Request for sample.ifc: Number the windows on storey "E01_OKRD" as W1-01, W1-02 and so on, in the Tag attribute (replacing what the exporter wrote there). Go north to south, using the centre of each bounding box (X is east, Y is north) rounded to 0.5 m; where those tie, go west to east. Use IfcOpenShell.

First a look at what the model holds.

```python
import ifcopenshell
import ifcopenshell.util.element
import ifcopenshell.util.placement

model = ifcopenshell.open("sample.ifc")
print(model.schema)
storey = next(s for s in model.by_type("IfcBuildingStorey") if s.Name == "E01_OKRD")
windows = [e for e in ifcopenshell.util.element.get_decomposition(storey) if e.is_a("IfcWindow")]
for e in sorted(windows, key=lambda e: e.id()):
    origin = ifcopenshell.util.placement.get_local_placement(e.ObjectPlacement)[:3, 3]
    print(e.id(), e.Tag, e.Name, origin.round(2) + 0.0, sep=" | ")
```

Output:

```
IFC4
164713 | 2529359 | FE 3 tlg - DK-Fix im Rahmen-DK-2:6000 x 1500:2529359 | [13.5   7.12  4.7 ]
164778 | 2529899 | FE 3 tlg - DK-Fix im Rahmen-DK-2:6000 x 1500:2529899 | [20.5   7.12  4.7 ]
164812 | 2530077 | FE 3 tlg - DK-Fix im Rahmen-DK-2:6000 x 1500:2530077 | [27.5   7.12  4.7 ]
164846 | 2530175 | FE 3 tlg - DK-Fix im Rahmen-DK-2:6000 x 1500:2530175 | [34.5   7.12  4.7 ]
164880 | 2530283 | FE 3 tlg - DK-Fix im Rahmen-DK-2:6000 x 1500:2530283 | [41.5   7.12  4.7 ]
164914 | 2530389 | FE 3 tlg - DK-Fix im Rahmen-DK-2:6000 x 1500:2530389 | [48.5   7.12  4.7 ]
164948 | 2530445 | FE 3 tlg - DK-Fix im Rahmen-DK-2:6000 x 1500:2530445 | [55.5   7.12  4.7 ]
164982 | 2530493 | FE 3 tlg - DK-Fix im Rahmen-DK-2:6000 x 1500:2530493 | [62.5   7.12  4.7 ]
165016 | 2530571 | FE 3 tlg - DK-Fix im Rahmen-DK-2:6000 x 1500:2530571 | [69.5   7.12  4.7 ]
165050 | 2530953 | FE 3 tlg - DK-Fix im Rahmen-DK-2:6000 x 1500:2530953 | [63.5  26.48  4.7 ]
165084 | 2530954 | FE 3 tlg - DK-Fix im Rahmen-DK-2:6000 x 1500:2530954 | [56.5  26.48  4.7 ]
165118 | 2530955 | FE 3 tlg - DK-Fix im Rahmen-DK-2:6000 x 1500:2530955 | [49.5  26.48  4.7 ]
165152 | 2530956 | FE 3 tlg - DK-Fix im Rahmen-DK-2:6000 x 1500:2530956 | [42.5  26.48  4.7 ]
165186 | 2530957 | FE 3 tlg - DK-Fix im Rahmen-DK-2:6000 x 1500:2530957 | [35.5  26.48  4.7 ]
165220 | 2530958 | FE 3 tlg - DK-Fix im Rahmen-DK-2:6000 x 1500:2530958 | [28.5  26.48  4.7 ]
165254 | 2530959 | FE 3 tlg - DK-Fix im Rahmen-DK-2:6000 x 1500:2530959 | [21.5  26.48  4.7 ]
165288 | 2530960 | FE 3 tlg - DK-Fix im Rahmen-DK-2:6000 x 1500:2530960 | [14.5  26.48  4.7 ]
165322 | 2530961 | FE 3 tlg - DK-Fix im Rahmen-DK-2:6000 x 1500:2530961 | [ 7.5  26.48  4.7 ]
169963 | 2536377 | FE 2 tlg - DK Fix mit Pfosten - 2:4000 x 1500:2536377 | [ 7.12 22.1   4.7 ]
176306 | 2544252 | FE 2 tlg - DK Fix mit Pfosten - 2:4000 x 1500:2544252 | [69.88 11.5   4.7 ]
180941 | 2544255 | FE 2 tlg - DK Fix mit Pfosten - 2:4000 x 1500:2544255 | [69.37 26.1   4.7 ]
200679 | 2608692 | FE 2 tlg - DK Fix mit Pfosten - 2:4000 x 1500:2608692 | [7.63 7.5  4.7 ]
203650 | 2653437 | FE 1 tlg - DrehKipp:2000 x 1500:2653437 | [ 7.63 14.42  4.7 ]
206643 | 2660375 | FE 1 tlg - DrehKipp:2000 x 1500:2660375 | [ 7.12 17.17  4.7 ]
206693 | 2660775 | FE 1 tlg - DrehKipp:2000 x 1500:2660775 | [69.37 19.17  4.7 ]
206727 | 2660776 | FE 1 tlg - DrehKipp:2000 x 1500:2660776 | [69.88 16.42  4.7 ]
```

```python
import ifcopenshell
import ifcopenshell.geom
import ifcopenshell.util.element
import ifcopenshell.util.shape

model = ifcopenshell.open("sample.ifc")
settings = ifcopenshell.geom.settings()
settings.set("use-world-coords", True)


def centre(element):
    shape = ifcopenshell.geom.create_shape(settings, element)
    return ifcopenshell.util.shape.get_bbox_centroid(shape.geometry)


storey = next(s for s in model.by_type("IfcBuildingStorey") if s.Name == "E01_OKRD")
windows = [e for e in ifcopenshell.util.element.get_decomposition(storey) if e.is_a("IfcWindow")]

# Insertion points can sit at a corner or the storey origin, so sort by the geometry (in metres).
centres = {e: centre(e) for e in windows}
windows.sort(key=lambda e: (-round(centres[e][1] / 0.5), centres[e][0]))

for i, e in enumerate(windows, start=1):
    number = f"W1-{i:02d}"
    e.Tag = number
    print(e.id(), number)

model.write("sample_edited.ifc")
```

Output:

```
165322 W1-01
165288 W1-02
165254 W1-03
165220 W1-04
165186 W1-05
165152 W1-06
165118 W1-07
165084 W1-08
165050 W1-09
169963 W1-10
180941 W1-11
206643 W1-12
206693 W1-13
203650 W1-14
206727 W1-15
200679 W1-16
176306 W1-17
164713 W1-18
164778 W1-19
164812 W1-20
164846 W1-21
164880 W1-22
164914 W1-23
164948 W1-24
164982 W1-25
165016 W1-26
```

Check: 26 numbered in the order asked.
